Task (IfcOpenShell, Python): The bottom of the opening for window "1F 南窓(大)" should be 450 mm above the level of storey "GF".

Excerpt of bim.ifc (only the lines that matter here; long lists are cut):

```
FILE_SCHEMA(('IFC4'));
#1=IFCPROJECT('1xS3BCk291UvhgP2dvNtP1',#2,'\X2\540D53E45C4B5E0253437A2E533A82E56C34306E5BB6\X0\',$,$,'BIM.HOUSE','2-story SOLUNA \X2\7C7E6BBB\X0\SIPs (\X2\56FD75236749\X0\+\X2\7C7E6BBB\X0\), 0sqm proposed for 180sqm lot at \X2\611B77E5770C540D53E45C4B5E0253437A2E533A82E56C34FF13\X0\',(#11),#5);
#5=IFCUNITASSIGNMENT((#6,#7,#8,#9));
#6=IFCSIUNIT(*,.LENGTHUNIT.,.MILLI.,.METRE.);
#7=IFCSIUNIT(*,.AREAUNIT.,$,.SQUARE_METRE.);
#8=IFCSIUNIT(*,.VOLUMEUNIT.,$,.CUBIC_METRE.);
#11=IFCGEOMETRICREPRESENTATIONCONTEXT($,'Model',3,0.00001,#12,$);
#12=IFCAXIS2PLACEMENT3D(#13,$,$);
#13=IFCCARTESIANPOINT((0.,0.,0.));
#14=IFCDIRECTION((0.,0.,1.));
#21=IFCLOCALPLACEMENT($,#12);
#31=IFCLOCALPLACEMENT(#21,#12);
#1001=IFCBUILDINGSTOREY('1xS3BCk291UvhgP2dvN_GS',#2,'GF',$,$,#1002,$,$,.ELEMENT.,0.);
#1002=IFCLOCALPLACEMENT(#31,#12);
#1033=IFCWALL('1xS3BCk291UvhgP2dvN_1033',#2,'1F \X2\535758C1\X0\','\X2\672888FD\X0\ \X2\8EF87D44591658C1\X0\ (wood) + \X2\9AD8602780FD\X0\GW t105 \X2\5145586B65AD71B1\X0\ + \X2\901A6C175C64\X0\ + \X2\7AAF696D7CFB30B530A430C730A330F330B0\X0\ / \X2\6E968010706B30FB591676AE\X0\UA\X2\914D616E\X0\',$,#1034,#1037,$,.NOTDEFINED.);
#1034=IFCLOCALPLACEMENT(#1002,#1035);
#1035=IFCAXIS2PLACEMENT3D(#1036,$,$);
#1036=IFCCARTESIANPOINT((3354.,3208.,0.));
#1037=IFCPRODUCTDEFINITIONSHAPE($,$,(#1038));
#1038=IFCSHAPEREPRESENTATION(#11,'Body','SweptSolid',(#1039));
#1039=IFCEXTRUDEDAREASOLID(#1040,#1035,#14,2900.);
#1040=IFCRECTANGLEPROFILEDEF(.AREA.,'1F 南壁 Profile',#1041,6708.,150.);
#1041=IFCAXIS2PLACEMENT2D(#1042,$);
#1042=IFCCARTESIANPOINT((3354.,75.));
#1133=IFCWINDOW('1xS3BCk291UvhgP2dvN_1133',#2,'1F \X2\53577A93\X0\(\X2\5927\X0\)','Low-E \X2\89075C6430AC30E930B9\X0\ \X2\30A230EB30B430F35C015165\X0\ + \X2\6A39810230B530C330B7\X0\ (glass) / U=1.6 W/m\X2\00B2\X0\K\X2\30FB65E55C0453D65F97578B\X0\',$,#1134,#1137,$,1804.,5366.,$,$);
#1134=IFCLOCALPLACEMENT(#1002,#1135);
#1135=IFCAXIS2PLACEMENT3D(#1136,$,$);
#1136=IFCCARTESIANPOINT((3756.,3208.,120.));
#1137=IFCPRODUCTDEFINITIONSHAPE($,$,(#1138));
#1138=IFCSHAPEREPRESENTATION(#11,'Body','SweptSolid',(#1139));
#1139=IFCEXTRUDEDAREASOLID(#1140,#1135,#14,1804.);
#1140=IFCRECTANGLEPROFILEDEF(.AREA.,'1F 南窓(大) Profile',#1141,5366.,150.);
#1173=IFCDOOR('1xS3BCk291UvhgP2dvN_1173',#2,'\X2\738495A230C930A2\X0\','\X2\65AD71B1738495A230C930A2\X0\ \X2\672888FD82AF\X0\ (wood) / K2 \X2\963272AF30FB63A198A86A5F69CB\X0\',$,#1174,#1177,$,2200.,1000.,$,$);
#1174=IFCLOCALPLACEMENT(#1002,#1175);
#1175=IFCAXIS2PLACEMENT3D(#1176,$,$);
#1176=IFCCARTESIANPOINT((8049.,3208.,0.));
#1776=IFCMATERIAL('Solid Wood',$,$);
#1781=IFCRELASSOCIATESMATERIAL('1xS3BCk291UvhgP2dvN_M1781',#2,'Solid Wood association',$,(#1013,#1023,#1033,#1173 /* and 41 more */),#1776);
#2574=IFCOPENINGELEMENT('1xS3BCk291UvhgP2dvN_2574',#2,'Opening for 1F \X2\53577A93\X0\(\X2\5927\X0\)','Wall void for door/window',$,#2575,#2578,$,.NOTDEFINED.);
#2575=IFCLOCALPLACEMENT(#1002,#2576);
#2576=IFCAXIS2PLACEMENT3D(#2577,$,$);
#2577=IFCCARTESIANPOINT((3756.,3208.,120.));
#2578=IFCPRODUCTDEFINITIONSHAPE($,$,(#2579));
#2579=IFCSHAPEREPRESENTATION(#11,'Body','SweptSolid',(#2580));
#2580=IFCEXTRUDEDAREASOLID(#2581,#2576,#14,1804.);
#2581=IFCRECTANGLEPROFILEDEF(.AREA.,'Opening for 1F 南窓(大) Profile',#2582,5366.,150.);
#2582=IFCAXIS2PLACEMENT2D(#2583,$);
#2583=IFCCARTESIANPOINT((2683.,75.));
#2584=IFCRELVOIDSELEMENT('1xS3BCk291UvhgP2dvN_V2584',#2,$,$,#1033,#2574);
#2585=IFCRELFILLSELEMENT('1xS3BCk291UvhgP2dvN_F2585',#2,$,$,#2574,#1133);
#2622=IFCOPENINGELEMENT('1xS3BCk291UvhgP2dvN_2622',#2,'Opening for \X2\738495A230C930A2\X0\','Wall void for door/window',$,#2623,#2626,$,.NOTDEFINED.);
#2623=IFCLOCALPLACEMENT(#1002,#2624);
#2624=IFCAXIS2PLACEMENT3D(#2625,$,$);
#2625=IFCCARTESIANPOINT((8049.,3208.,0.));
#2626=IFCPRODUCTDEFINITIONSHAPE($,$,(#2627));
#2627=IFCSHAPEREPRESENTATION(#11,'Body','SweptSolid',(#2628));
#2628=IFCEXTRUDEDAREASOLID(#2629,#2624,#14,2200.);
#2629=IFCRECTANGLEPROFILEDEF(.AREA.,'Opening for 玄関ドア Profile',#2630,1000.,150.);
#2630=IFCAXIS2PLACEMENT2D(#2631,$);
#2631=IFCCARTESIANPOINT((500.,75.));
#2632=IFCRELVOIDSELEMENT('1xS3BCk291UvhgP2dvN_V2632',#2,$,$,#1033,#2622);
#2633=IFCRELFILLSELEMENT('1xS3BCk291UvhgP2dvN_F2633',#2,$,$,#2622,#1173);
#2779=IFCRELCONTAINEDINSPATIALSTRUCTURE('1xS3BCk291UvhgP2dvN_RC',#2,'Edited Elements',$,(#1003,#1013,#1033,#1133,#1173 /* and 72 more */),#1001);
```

```python
import numpy as np
import ifcopenshell
import ifcopenshell.api.geometry
import ifcopenshell.geom
import ifcopenshell.util.element
import ifcopenshell.util.placement
import ifcopenshell.util.shape
import ifcopenshell.util.unit

model = ifcopenshell.open("bim.ifc")
unit_scale = ifcopenshell.util.unit.calculate_unit_scale(model)

window = model.by_id(1133)
opening = window.FillsVoids[0].RelatingOpeningElement
storey = ifcopenshell.util.element.get_container(window, ifc_class="IfcBuildingStorey")
level = ifcopenshell.util.placement.get_local_placement(storey.ObjectPlacement)[2, 3]

# The opening's origin need not be at the sill, so measure its lowest point.
shape = ifcopenshell.geom.create_shape(ifcopenshell.geom.settings(), opening)
bottom = ifcopenshell.util.shape.get_shape_bottom_elevation(shape, shape.geometry) / unit_scale
dz = level + 0.45 / unit_scale - bottom

shift = np.array([0.0, 0.0, dz])
# The window is not placed relative to its opening, so move both.
for product in (opening, window):
    matrix = ifcopenshell.util.placement.get_local_placement(product.ObjectPlacement)
    matrix[:3, 3] += shift
    ifcopenshell.api.geometry.edit_object_placement(model, product=product, matrix=matrix, is_si=False)

print(f"moved by {dz * unit_scale:+.3f} m")

model.write("bim_updated.ifc")
```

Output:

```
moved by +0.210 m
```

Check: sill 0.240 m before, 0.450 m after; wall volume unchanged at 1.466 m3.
